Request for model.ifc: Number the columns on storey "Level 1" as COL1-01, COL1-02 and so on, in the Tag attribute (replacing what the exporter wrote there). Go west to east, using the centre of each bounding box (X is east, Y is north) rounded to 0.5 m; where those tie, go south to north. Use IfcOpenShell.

First a look at what the model holds.

```python
import ifcopenshell
import ifcopenshell.util.element
import ifcopenshell.util.placement

model = ifcopenshell.open("model.ifc")
print(model.schema)
storey = next(s for s in model.by_type("IfcBuildingStorey") if s.Name == "Level 1")
columns = [e for e in ifcopenshell.util.element.get_decomposition(storey) if e.is_a("IfcColumn")]
for e in sorted(columns, key=lambda e: e.id()):
    origin = ifcopenshell.util.placement.get_local_placement(e.ObjectPlacement)[:3, 3]
    print(e.id(), e.Tag, e.Name, origin.round(2) + 0.0, sep=" | ")
```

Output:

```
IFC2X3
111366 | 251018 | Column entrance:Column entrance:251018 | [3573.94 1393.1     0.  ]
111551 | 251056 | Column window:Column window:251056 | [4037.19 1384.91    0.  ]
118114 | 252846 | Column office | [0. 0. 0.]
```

```python
import ifcopenshell
import ifcopenshell.geom
import ifcopenshell.util.element
import ifcopenshell.util.shape

model = ifcopenshell.open("model.ifc")
settings = ifcopenshell.geom.settings()
settings.set("use-world-coords", True)


def centre(element):
    shape = ifcopenshell.geom.create_shape(settings, element)
    return ifcopenshell.util.shape.get_bbox_centroid(shape.geometry)


storey = next(s for s in model.by_type("IfcBuildingStorey") if s.Name == "Level 1")
columns = [e for e in ifcopenshell.util.element.get_decomposition(storey) if e.is_a("IfcColumn")]

# Insertion points can sit at a corner or the storey origin, so sort by the geometry (in metres).
centres = {e: centre(e) for e in columns}
columns.sort(key=lambda e: (round(centres[e][0] / 0.5), centres[e][1]))

for i, e in enumerate(columns, start=1):
    number = f"COL1-{i:02d}"
    e.Tag = number
    print(e.id(), number)

model.write("model_updated.ifc")
```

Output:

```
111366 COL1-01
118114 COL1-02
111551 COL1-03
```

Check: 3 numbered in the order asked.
